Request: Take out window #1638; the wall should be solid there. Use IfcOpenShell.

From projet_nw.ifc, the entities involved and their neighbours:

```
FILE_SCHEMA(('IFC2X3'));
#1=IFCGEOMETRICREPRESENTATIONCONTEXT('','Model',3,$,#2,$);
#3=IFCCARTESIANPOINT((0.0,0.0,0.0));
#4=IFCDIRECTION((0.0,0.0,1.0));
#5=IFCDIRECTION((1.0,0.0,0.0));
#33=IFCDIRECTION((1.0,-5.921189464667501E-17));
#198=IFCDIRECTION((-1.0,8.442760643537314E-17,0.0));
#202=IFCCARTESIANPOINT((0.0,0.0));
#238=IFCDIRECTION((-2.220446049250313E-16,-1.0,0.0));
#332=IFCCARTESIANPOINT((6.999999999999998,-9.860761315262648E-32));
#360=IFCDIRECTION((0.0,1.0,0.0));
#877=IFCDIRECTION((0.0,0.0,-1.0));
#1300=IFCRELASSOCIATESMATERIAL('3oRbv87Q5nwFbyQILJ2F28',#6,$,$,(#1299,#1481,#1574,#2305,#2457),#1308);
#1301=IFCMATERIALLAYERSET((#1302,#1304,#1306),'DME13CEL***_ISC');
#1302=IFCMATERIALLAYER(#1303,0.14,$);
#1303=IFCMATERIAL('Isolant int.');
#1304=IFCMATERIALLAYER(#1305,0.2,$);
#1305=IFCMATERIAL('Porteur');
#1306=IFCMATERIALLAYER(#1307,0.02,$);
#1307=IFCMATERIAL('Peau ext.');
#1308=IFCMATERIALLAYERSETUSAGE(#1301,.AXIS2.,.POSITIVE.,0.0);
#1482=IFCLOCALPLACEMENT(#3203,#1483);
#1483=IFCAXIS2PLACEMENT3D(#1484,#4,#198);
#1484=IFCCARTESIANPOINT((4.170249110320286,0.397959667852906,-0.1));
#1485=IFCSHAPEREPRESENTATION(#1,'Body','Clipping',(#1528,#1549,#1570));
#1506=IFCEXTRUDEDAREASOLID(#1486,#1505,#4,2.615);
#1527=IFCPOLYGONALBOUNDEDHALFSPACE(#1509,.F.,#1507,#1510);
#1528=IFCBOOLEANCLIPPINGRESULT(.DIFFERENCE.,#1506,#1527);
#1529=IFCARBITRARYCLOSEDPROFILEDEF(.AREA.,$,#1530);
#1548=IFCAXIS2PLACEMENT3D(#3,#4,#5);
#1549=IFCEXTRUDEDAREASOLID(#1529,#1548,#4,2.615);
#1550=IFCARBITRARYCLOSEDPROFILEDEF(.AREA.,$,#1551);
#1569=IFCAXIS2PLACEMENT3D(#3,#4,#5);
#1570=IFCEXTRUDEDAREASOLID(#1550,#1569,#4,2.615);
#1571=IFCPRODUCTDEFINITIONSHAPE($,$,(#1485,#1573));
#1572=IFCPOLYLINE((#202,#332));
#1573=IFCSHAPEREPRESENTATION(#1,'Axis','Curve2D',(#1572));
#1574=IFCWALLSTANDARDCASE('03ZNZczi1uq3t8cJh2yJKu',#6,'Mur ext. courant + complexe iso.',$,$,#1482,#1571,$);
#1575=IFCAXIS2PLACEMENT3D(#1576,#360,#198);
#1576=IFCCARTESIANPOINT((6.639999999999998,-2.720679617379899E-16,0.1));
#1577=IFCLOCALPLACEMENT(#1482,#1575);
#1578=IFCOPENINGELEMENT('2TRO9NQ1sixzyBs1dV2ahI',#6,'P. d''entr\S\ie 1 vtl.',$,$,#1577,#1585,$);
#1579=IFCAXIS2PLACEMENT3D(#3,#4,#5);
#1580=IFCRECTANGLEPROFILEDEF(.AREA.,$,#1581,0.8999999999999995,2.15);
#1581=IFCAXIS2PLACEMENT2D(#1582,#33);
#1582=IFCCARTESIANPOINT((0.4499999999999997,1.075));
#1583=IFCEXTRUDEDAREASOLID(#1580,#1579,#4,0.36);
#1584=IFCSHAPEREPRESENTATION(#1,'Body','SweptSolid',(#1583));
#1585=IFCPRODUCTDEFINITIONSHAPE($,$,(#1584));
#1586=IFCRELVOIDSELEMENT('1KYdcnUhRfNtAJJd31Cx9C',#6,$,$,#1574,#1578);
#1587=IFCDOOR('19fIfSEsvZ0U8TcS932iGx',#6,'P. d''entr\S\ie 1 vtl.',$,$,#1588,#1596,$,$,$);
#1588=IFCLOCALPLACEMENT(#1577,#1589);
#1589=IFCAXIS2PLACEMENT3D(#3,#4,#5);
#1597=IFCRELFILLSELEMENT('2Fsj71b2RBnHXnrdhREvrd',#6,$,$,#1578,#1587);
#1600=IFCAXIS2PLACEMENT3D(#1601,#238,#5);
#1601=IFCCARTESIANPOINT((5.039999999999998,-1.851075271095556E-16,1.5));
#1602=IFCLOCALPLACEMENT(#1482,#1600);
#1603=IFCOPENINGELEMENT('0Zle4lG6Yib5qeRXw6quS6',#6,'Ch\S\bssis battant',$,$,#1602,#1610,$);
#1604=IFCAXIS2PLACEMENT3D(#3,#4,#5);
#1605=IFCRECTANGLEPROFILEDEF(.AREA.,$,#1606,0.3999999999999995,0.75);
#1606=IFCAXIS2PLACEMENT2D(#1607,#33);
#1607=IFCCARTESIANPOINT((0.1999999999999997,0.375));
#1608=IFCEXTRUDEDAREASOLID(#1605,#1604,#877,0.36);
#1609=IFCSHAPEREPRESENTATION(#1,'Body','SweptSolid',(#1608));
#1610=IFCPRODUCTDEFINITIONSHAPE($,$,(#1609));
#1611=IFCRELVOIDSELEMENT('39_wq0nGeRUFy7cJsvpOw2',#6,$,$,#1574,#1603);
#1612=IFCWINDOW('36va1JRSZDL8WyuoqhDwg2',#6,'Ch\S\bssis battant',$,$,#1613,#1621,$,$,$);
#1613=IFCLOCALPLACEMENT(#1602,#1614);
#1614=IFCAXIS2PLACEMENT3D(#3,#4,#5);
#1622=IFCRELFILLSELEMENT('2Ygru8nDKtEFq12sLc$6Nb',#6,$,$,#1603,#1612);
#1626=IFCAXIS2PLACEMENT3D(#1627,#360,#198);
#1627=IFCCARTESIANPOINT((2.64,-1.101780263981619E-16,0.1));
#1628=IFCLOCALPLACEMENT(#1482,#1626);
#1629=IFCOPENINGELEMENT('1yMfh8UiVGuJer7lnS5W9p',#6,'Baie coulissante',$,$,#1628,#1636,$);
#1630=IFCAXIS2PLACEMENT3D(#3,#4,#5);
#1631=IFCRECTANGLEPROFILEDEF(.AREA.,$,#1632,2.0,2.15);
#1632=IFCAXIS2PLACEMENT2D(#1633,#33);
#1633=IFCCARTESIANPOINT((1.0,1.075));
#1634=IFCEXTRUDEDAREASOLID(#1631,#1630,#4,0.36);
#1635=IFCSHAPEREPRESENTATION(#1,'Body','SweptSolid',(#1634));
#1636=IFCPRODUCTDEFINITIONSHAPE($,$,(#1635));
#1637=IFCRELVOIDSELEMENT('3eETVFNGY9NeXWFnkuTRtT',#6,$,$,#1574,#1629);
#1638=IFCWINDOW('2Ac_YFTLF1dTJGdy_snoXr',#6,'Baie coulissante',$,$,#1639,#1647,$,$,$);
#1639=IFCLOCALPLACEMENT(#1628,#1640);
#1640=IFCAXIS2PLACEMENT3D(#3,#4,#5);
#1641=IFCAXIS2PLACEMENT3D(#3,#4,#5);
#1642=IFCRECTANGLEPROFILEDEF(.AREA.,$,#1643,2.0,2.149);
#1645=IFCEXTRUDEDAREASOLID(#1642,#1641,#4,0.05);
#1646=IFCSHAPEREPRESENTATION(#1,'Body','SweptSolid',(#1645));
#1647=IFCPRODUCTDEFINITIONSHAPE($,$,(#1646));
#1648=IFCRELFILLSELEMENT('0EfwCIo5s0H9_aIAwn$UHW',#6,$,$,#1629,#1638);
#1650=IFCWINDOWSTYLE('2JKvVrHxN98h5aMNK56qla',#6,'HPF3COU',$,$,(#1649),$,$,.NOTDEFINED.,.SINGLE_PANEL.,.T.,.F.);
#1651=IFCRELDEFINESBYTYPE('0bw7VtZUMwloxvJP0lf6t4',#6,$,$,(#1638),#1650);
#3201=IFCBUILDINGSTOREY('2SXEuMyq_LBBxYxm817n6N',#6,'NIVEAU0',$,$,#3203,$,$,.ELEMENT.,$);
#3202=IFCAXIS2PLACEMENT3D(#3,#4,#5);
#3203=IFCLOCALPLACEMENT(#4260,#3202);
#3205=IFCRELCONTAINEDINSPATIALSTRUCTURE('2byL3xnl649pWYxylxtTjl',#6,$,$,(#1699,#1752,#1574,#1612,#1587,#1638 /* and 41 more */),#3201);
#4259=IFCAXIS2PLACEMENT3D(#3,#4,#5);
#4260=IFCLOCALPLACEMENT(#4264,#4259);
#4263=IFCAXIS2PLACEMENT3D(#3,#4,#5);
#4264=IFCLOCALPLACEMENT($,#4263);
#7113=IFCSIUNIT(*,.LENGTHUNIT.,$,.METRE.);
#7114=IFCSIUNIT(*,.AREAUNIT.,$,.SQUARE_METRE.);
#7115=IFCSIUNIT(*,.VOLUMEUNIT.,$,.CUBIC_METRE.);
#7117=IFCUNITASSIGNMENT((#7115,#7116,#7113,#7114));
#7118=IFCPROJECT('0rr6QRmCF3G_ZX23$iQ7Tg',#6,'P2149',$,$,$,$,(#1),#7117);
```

```python
import ifcopenshell
import ifcopenshell.api.feature
import ifcopenshell.api.root
import ifcopenshell.geom
import ifcopenshell.util.shape

model = ifcopenshell.open("projet_nw.ifc")
settings = ifcopenshell.geom.settings()


def volume(element):
    """Net volume in cubic metres, openings subtracted."""
    shape = ifcopenshell.geom.create_shape(settings, element)
    return ifcopenshell.util.shape.get_volume(shape.geometry)


window = model.by_guid("2Ac_YFTLF1dTJGdy_snoXr")
opening = window.FillsVoids[0].RelatingOpeningElement
wall = opening.VoidsElements[0].RelatingBuildingElement
before = volume(wall)

ifcopenshell.api.root.remove_product(model, product=window)
ifcopenshell.api.feature.remove_feature(model, feature=opening)

after = volume(wall)

print(f"wall volume {before:.3f} -> {after:.3f} m3")

model.write("projet_nw_v2.ifc")
```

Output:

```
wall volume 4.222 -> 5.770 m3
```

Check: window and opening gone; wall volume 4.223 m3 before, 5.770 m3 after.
